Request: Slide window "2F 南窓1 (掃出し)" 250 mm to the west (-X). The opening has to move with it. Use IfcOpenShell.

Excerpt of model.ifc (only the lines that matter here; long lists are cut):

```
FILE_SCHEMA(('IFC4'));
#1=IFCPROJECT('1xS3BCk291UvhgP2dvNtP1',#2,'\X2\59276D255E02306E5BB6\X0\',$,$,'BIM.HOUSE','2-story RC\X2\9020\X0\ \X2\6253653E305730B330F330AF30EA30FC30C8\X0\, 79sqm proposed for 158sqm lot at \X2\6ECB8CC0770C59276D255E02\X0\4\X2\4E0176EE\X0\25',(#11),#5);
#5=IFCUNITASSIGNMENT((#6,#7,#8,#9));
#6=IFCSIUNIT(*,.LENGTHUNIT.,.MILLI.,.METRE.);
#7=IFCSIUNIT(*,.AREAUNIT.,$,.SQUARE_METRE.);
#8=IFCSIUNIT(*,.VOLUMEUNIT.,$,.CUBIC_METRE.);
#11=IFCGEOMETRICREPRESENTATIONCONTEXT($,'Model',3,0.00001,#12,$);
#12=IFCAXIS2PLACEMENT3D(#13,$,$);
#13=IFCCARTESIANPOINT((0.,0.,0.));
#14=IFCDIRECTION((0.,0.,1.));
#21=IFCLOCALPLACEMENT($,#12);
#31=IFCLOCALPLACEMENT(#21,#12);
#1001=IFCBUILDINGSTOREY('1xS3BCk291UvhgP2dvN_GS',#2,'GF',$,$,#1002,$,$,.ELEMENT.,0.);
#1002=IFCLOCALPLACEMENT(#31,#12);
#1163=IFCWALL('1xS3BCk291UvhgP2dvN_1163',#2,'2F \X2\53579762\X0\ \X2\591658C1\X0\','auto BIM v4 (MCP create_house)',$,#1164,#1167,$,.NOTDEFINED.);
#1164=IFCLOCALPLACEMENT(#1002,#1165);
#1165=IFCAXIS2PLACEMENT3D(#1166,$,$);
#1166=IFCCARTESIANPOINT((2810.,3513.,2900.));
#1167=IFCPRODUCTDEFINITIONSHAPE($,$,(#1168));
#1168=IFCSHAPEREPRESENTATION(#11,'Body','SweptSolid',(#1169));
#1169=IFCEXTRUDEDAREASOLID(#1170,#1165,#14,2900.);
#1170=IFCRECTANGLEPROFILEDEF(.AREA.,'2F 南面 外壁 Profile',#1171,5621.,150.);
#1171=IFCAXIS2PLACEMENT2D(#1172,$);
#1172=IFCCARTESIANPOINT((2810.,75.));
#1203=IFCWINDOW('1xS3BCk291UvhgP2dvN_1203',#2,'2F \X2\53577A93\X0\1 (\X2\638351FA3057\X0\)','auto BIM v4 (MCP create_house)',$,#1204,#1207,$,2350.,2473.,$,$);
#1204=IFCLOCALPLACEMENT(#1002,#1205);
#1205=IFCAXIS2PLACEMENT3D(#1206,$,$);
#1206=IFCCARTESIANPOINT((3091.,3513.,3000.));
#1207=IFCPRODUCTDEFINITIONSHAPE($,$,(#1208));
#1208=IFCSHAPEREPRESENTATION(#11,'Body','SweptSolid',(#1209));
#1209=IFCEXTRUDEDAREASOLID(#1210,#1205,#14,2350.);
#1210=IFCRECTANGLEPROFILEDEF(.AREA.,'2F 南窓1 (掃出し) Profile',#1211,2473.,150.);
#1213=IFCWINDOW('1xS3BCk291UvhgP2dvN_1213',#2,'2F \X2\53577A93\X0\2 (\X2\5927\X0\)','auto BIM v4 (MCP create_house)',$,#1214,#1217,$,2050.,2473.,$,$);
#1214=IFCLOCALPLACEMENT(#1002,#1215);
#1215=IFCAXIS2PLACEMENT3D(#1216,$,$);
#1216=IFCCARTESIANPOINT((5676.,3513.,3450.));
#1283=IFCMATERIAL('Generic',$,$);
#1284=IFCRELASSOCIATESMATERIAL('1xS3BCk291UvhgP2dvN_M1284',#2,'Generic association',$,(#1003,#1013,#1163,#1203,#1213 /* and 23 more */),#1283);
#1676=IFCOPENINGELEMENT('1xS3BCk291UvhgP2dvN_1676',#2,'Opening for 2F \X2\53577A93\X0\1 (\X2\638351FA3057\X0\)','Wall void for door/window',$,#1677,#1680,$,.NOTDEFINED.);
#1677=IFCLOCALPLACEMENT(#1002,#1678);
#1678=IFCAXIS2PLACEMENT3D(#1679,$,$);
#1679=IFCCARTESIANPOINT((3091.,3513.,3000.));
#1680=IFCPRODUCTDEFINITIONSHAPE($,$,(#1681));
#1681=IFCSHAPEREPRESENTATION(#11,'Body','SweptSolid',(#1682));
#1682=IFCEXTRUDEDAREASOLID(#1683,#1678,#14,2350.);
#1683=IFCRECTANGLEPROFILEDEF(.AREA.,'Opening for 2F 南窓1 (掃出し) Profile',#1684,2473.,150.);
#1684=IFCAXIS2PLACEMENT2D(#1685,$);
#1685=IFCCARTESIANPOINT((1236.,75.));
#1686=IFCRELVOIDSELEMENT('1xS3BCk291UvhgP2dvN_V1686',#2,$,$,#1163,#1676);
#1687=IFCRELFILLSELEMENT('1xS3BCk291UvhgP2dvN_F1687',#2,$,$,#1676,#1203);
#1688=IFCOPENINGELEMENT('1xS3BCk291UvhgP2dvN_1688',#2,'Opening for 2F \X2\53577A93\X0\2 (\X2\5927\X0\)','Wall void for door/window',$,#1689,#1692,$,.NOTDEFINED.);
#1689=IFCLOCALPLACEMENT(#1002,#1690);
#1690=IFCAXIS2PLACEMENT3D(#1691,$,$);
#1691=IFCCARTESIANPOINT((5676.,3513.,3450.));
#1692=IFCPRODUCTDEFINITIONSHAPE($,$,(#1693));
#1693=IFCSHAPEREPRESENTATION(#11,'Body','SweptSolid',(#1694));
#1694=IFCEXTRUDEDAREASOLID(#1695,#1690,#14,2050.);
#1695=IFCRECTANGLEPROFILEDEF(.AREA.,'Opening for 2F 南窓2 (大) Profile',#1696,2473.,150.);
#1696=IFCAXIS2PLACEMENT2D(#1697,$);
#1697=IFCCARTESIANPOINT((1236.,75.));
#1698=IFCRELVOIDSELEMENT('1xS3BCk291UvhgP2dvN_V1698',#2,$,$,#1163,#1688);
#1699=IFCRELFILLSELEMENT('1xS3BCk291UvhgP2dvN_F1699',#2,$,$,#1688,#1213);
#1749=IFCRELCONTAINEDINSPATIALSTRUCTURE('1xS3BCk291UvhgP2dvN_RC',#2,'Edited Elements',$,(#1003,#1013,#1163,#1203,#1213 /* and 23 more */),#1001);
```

```python
import ifcopenshell
import ifcopenshell.api.geometry
import ifcopenshell.util.placement
import ifcopenshell.util.unit

model = ifcopenshell.open("model.ifc")
unit_scale = ifcopenshell.util.unit.calculate_unit_scale(model)

window = model.by_guid("1xS3BCk291UvhgP2dvN_1203")
opening = window.FillsVoids[0].RelatingOpeningElement
wall = opening.VoidsElements[0].RelatingBuildingElement

wall_matrix = ifcopenshell.util.placement.get_local_placement(wall.ObjectPlacement)
shift = wall_matrix[:3, 0] * -0.25 / unit_scale
before = ifcopenshell.util.placement.get_local_placement(window.ObjectPlacement)[:3, 3].copy()

# The window is not placed relative to its opening, so move both.
for product in (opening, window):
    matrix = ifcopenshell.util.placement.get_local_placement(product.ObjectPlacement)
    matrix[:3, 3] += shift
    ifcopenshell.api.geometry.edit_object_placement(model, product=product, matrix=matrix, is_si=False)

after = ifcopenshell.util.placement.get_local_placement(window.ObjectPlacement)[:3, 3]
print("window moved by", (after - before).round(3) + 0.0)

model.write("model_v2.ifc")
```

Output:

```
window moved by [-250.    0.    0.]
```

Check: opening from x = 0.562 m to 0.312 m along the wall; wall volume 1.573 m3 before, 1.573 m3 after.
